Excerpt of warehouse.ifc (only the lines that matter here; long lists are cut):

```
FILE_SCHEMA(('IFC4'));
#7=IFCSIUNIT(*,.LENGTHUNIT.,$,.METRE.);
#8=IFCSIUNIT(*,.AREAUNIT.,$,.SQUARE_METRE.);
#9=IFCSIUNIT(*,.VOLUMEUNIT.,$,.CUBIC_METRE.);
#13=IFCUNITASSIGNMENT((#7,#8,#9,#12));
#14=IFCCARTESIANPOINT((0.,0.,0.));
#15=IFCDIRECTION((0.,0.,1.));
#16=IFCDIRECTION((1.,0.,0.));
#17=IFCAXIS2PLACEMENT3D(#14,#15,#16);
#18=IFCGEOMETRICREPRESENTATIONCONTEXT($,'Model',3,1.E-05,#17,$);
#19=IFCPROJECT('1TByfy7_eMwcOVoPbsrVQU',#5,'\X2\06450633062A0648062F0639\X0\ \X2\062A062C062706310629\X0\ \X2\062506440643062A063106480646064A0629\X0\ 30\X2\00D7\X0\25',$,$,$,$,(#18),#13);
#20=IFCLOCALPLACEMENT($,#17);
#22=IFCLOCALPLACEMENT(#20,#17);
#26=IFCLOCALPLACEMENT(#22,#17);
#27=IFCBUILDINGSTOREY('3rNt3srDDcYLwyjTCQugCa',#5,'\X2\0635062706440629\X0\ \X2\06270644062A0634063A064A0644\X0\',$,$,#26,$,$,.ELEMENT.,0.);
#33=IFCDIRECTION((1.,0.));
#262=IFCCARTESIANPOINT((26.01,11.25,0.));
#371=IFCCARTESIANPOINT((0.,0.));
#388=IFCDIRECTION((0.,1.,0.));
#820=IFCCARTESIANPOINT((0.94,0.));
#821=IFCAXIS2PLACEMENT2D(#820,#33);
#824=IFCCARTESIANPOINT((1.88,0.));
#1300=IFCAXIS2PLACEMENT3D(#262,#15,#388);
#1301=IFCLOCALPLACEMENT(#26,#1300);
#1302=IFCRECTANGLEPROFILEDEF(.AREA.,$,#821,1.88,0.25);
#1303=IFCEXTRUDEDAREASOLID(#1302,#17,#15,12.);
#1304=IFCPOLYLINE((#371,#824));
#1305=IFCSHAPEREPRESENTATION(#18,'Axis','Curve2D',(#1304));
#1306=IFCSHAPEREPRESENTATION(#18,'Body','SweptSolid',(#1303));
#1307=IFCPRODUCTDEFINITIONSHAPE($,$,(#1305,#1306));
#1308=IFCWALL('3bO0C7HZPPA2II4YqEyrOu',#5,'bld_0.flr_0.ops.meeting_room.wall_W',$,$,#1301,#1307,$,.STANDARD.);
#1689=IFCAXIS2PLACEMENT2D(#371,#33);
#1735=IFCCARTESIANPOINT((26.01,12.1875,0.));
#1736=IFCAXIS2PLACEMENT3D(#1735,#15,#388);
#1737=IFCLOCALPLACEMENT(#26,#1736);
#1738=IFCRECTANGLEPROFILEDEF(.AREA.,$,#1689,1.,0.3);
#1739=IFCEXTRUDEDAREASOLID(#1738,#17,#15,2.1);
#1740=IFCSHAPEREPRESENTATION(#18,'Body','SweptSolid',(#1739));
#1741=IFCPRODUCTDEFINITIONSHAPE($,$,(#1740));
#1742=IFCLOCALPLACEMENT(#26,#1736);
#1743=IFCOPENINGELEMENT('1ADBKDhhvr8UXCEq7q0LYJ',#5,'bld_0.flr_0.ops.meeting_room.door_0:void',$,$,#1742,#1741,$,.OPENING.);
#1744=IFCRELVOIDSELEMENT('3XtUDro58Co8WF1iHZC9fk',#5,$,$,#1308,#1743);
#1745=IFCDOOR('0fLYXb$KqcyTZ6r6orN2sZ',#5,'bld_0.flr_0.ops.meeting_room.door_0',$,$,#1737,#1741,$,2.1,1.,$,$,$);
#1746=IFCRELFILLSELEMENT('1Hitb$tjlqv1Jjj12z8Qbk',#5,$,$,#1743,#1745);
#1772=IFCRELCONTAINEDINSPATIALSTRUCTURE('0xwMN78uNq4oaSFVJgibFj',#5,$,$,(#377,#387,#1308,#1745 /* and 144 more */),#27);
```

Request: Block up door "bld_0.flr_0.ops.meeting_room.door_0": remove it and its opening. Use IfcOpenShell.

```python
import ifcopenshell
import ifcopenshell.api.feature
import ifcopenshell.api.root
import ifcopenshell.geom
import ifcopenshell.util.shape

model = ifcopenshell.open("warehouse.ifc")
settings = ifcopenshell.geom.settings()


def volume(element):
    """Net volume in cubic metres, openings subtracted."""
    shape = ifcopenshell.geom.create_shape(settings, element)
    return ifcopenshell.util.shape.get_volume(shape.geometry)


door = model.by_guid("0fLYXb$KqcyTZ6r6orN2sZ")
opening = door.FillsVoids[0].RelatingOpeningElement
wall = opening.VoidsElements[0].RelatingBuildingElement
before = volume(wall)

ifcopenshell.api.root.remove_product(model, product=door)
ifcopenshell.api.feature.remove_feature(model, feature=opening)

after = volume(wall)

print(f"wall volume {before:.3f} -> {after:.3f} m3")

model.write("warehouse_updated.ifc")
```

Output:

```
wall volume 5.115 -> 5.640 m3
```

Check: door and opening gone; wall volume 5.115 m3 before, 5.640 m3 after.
